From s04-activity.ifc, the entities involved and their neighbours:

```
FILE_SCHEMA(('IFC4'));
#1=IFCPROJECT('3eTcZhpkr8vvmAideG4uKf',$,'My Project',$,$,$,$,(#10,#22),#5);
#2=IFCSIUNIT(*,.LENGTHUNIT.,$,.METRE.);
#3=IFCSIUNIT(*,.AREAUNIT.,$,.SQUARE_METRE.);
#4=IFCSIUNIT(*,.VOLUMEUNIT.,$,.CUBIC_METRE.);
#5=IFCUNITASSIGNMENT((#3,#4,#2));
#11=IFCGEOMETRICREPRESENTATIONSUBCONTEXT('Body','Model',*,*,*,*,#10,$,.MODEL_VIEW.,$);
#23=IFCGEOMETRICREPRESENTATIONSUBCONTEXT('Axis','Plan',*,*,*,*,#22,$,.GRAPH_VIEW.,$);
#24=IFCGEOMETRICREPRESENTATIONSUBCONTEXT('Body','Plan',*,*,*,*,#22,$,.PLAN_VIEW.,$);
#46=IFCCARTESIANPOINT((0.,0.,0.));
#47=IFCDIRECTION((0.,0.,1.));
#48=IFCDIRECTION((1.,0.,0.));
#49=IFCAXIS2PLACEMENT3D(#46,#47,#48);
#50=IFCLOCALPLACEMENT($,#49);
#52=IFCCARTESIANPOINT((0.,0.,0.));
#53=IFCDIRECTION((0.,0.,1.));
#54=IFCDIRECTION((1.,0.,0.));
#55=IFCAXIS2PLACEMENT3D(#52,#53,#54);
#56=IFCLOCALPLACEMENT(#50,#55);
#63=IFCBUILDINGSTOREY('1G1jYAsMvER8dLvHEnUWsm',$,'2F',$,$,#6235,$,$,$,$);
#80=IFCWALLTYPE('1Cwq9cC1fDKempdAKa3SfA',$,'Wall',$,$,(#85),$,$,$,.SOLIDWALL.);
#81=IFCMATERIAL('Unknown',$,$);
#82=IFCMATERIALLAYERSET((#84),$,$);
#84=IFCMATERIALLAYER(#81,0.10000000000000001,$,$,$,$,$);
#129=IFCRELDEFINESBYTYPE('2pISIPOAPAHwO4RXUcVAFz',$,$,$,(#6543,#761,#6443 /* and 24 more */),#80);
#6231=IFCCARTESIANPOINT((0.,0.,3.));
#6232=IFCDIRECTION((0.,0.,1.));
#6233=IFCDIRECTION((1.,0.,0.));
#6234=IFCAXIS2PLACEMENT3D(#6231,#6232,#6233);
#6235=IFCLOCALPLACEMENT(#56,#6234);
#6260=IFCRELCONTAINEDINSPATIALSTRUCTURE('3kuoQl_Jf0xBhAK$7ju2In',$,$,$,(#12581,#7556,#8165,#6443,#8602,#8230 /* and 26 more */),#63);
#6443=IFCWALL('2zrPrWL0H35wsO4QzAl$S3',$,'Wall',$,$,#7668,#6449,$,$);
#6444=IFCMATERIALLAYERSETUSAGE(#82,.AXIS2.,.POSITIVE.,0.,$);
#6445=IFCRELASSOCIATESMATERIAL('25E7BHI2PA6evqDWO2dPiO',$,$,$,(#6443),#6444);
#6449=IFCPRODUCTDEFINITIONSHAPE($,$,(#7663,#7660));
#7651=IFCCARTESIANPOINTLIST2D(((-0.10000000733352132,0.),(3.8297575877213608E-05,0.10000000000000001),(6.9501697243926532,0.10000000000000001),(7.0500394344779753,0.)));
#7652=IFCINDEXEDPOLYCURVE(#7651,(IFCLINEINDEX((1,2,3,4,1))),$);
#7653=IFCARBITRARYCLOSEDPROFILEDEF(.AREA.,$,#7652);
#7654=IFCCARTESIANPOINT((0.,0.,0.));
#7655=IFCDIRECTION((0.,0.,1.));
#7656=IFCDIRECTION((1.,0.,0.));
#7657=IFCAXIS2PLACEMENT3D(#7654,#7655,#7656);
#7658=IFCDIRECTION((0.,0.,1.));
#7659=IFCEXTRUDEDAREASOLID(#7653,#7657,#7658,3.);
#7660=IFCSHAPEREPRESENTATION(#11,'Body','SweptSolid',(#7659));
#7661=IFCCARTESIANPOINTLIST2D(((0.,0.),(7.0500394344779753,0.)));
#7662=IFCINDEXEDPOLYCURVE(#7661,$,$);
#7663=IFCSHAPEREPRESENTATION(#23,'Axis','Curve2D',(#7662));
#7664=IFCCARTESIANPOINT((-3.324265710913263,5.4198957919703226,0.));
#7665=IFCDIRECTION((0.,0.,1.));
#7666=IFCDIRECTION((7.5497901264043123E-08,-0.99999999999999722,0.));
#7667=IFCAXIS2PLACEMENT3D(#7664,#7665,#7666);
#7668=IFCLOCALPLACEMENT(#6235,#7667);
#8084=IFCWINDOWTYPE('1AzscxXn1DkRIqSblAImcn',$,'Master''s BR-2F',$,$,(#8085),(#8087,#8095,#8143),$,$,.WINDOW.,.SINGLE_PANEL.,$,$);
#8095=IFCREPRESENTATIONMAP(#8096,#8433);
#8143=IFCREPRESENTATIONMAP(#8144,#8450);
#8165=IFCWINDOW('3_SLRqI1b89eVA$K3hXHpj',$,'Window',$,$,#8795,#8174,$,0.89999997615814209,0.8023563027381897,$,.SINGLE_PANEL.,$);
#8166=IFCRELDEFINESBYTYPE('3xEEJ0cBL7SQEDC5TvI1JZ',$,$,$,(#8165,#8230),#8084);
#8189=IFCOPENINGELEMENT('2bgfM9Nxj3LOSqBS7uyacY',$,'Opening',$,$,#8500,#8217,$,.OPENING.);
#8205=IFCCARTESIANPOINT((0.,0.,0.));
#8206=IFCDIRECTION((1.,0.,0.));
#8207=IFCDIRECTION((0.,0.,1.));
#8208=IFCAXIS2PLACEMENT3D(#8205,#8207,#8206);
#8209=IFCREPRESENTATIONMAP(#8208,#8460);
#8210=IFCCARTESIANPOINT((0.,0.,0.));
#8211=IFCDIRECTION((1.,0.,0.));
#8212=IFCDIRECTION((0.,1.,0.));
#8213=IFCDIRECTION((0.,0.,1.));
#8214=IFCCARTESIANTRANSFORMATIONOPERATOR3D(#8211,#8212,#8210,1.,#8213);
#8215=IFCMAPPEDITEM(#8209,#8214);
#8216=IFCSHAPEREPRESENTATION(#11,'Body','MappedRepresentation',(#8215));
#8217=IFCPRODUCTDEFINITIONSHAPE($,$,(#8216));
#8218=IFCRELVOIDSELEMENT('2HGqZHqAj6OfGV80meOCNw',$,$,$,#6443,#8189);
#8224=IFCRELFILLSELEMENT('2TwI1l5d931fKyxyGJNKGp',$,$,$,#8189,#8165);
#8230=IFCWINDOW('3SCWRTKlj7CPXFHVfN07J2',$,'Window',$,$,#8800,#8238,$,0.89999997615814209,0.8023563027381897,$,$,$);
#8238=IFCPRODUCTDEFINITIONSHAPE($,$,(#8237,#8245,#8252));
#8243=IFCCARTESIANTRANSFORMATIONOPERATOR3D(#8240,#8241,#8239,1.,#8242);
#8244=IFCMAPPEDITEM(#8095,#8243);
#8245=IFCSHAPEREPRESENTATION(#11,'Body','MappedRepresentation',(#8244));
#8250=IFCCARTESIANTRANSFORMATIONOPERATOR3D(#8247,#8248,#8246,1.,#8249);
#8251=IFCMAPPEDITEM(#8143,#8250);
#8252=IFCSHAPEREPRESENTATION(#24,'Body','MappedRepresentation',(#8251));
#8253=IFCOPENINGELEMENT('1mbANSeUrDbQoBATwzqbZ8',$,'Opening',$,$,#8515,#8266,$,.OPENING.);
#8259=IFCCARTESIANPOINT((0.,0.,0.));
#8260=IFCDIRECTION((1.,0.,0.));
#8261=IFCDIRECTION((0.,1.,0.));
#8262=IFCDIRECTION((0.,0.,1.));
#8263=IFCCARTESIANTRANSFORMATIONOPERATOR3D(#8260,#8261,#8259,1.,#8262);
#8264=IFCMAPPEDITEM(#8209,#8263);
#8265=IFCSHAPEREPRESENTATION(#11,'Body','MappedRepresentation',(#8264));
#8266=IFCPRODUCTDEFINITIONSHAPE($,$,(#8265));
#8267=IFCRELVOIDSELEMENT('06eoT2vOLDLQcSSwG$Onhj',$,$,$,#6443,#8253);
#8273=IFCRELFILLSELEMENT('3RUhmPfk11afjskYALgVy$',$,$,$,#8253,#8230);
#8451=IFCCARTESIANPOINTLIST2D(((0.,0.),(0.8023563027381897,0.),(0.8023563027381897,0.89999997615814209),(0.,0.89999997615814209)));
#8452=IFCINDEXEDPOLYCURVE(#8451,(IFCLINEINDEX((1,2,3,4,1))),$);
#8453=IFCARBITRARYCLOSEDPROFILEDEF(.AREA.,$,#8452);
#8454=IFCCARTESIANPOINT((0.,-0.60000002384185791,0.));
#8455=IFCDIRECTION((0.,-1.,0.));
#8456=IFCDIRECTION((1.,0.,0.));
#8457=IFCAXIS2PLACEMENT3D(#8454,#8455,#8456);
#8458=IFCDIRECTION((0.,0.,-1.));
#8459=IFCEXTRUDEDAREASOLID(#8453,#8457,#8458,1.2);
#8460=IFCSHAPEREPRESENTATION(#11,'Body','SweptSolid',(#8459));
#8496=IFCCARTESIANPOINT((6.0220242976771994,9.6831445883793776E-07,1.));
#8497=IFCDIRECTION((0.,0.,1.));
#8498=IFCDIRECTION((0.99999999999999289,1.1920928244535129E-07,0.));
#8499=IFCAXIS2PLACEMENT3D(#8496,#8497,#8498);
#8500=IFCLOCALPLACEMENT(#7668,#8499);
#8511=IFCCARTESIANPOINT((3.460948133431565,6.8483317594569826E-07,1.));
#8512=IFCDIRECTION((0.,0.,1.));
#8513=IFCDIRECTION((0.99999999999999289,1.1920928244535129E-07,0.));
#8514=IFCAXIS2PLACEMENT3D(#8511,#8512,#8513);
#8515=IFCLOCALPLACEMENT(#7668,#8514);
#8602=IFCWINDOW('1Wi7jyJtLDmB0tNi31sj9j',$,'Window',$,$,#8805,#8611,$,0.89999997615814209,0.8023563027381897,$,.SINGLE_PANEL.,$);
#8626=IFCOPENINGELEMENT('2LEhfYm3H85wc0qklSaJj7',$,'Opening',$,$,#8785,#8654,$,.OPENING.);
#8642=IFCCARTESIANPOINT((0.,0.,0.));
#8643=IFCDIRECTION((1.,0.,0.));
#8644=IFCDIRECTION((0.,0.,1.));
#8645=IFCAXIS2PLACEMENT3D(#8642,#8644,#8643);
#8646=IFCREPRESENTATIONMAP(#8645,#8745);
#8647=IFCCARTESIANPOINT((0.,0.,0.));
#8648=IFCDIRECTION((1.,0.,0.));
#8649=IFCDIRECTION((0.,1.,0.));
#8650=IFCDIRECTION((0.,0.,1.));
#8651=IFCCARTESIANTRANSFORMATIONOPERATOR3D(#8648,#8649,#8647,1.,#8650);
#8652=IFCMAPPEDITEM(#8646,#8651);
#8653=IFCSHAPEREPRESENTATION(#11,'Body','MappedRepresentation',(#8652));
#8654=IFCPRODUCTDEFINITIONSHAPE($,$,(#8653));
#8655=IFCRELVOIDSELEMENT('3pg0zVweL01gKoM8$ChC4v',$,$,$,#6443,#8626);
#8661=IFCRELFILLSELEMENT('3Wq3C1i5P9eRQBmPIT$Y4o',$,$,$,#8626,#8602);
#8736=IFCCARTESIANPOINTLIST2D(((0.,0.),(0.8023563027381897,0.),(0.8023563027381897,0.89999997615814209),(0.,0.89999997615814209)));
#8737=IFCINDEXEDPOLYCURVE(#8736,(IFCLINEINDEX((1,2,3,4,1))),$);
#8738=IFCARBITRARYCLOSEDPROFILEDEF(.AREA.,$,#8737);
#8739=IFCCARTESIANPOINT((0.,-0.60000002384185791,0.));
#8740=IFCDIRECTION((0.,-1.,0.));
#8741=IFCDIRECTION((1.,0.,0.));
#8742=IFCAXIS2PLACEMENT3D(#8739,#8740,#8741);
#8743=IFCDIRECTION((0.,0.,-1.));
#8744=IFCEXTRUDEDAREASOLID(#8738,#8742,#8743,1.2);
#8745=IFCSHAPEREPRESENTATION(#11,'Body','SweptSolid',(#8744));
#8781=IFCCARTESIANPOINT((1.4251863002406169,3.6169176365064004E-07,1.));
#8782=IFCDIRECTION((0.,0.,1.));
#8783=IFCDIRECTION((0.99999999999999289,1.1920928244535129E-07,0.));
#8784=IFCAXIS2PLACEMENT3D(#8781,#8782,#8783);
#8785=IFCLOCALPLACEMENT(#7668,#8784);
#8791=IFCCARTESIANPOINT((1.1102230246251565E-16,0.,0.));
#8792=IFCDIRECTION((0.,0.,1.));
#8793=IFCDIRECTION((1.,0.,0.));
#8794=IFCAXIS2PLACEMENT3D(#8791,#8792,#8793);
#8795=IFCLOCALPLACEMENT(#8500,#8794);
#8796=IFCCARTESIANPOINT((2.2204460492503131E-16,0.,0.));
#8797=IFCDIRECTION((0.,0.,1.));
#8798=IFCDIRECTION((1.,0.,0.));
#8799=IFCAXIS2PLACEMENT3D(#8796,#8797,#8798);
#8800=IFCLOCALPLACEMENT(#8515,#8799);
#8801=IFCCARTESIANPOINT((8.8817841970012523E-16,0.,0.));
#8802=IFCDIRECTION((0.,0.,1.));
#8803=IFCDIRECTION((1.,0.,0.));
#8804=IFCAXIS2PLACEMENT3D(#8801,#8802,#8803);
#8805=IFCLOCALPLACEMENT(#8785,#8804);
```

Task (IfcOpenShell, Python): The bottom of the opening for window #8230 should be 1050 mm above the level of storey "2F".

```python
import numpy as np
import ifcopenshell
import ifcopenshell.api.geometry
import ifcopenshell.geom
import ifcopenshell.util.element
import ifcopenshell.util.placement
import ifcopenshell.util.shape
import ifcopenshell.util.unit

model = ifcopenshell.open("s04-activity.ifc")
unit_scale = ifcopenshell.util.unit.calculate_unit_scale(model)

window = model.by_guid("3SCWRTKlj7CPXFHVfN07J2")
opening = window.FillsVoids[0].RelatingOpeningElement
storey = ifcopenshell.util.element.get_container(window, ifc_class="IfcBuildingStorey")
level = ifcopenshell.util.placement.get_local_placement(storey.ObjectPlacement)[2, 3]

# The opening's origin need not be at the sill, so measure its lowest point.
shape = ifcopenshell.geom.create_shape(ifcopenshell.geom.settings(), opening)
bottom = ifcopenshell.util.shape.get_shape_bottom_elevation(shape, shape.geometry) / unit_scale
dz = level + 1.05 / unit_scale - bottom

shift = np.array([0.0, 0.0, dz])
# The window is placed relative to its opening, so it follows when the opening moves.
matrix = ifcopenshell.util.placement.get_local_placement(opening.ObjectPlacement)
matrix[:3, 3] += shift
ifcopenshell.api.geometry.edit_object_placement(
    model, product=opening, matrix=matrix, is_si=False, should_transform_children=True
)

print(f"moved by {dz * unit_scale:+.3f} m")

model.write("s04-activity-out.ifc")
```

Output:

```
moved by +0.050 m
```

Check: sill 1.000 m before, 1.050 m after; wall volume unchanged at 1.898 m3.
